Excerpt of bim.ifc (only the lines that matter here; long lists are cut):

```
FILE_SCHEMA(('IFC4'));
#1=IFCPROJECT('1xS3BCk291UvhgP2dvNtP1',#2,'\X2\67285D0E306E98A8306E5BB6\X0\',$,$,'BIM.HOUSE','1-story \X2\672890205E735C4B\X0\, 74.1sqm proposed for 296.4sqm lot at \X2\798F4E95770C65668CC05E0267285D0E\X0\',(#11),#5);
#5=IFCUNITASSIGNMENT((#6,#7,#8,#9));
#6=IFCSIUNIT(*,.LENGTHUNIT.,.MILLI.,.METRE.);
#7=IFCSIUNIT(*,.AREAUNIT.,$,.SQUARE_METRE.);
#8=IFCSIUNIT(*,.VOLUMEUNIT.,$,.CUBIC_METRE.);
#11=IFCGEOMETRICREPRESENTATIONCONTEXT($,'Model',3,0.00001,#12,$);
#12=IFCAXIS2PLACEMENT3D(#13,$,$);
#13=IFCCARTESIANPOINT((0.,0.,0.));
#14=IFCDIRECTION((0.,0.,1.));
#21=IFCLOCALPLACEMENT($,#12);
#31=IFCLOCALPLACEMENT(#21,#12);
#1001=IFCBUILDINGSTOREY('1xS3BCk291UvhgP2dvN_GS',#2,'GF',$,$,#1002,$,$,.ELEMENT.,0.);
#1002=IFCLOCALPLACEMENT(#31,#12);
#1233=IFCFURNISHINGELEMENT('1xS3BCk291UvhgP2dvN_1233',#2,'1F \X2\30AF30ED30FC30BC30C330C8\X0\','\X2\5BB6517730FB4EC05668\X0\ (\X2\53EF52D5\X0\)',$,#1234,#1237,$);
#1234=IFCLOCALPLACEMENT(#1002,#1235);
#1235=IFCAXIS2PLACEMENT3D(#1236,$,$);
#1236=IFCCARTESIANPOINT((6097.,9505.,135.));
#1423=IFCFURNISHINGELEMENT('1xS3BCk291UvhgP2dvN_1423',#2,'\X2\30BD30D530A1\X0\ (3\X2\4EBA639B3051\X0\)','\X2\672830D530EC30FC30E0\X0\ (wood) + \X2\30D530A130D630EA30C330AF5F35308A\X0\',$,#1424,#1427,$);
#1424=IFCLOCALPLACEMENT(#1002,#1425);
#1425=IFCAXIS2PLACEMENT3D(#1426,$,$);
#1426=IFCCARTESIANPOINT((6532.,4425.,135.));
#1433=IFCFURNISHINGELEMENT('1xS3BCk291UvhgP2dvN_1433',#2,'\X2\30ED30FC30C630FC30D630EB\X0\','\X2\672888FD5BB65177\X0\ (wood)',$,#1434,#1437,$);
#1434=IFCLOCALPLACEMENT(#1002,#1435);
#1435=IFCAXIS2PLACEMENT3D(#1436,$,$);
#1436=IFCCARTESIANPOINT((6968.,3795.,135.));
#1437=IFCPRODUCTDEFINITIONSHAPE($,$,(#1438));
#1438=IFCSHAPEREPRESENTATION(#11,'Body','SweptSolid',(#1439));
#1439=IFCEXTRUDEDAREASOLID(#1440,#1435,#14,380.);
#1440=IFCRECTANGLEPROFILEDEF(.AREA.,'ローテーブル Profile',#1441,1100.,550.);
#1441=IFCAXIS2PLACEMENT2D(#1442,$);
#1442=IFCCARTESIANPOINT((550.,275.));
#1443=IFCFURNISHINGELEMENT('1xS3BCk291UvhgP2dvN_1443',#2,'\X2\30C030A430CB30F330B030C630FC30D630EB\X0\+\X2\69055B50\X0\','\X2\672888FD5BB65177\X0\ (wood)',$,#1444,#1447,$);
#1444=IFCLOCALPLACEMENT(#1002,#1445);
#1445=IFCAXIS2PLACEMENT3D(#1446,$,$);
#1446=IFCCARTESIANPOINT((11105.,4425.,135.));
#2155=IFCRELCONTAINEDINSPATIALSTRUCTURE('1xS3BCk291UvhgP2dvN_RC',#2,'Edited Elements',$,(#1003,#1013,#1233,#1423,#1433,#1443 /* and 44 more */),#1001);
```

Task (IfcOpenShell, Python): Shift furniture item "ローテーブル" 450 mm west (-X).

```python
import ifcopenshell
import ifcopenshell.api.geometry
import ifcopenshell.util.placement
import ifcopenshell.util.unit

model = ifcopenshell.open("bim.ifc")
unit_scale = ifcopenshell.util.unit.calculate_unit_scale(model)

item = model.by_guid("1xS3BCk291UvhgP2dvN_1433")
matrix = ifcopenshell.util.placement.get_local_placement(item.ObjectPlacement)
matrix[0, 3] -= 0.45 / unit_scale
ifcopenshell.api.geometry.edit_object_placement(model, product=item, matrix=matrix, is_si=False)

print(ifcopenshell.util.placement.get_local_placement(item.ObjectPlacement).round(3) + 0.0)

model.write("bim-out.ifc")
```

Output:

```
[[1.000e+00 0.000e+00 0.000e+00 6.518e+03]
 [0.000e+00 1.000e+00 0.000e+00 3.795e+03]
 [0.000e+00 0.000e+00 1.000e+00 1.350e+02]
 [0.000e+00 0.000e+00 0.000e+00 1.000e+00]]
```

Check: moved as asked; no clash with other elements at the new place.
